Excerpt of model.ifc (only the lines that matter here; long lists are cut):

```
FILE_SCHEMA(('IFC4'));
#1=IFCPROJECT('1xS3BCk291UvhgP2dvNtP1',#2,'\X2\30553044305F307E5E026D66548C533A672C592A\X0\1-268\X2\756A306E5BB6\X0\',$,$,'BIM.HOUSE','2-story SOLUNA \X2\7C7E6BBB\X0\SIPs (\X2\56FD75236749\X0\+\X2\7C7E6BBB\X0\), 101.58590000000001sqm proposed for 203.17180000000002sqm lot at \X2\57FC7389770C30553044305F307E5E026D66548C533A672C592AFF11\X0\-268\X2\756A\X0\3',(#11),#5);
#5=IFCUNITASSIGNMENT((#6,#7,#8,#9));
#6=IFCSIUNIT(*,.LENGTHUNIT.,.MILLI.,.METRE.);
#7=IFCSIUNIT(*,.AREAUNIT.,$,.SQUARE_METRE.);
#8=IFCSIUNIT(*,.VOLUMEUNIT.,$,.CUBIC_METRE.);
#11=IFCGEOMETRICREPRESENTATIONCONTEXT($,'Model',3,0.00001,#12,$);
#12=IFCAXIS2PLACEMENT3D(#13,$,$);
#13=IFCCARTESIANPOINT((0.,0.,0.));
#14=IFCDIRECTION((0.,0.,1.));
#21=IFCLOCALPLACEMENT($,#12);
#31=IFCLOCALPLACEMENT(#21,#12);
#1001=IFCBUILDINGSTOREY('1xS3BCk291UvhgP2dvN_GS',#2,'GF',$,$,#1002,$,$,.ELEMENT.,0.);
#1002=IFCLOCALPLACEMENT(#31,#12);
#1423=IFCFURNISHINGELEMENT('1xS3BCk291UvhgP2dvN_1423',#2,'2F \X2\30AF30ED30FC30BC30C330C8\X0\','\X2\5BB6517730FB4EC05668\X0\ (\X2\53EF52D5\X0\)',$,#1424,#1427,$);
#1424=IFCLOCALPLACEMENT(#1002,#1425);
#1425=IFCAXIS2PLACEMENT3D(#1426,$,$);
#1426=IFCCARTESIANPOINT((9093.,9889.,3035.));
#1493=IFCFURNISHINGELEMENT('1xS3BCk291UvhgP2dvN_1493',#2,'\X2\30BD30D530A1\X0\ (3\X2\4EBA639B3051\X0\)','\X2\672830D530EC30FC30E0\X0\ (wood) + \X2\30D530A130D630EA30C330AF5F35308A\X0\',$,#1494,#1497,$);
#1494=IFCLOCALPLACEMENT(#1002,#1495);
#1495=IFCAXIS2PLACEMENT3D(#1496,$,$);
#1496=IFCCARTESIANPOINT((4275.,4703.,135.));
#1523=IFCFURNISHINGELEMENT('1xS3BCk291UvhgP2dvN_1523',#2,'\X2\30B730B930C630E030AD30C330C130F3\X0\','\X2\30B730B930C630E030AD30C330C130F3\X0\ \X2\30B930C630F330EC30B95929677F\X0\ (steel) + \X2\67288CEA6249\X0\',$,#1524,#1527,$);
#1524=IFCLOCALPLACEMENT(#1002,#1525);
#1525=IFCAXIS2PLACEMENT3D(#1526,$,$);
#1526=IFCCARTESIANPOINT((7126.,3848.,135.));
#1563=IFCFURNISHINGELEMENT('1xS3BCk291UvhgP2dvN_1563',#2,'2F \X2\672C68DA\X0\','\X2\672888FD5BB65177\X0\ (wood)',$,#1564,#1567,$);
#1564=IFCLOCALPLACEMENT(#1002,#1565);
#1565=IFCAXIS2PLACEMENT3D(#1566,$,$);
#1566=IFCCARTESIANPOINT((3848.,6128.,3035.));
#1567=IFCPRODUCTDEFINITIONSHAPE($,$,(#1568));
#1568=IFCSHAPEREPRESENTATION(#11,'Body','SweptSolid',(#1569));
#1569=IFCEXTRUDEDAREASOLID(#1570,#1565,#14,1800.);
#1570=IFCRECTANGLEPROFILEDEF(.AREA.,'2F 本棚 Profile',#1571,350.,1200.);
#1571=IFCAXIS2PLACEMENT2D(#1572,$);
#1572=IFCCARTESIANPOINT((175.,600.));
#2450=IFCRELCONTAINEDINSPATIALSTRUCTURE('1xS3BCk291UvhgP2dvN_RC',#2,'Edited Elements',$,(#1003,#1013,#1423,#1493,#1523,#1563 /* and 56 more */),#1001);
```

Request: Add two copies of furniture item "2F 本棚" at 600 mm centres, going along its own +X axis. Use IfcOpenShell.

```python
import ifcopenshell
import ifcopenshell.api.geometry
import ifcopenshell.api.root
import ifcopenshell.util.element
import ifcopenshell.util.placement
import ifcopenshell.util.unit

model = ifcopenshell.open("model.ifc")
unit_scale = ifcopenshell.util.unit.calculate_unit_scale(model)


def reuse_history(source, copy):
    """copy_class also copies each property set's owner history, people and application; keep the originals."""
    for rel in copy.IsDefinedBy:
        if rel.is_a("IfcRelDefinesByProperties") and (history := rel.RelatingPropertyDefinition.OwnerHistory):
            rel.RelatingPropertyDefinition.OwnerHistory = source.OwnerHistory
            ifcopenshell.util.element.remove_deep2(model, history)


source = model.by_id(1563)
base = ifcopenshell.util.placement.get_local_placement(source.ObjectPlacement)
step = base[:3, 0] * 0.6 / unit_scale

for i in range(1, 3):
    copy = ifcopenshell.api.root.copy_class(model, product=source)
    copy.Representation = ifcopenshell.util.element.copy_deep(
        model, source.Representation, exclude=["IfcGeometricRepresentationContext", "IfcRepresentationMap"]
    )
    reuse_history(source, copy)
    matrix = base.copy()
    matrix[:3, 3] += i * step
    print("added at", matrix[:3, 3].round(3) + 0.0)
    ifcopenshell.api.geometry.edit_object_placement(model, product=copy, matrix=matrix, is_si=False)

model.write("model-out.ifc")
```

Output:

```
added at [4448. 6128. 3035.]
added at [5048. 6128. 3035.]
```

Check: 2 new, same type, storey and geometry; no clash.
